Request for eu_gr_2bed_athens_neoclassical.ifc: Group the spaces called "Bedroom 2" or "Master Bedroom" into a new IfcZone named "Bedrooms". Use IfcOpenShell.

First a look at what the model holds.

```python
import ifcopenshell

model = ifcopenshell.open("eu_gr_2bed_athens_neoclassical.ifc")
print(model.schema)
seen = {}
for space in model.by_type("IfcSpace"):
    seen[space.LongName] = seen.get(space.LongName, 0) + 1
for name, count in sorted(seen.items(), key=str):
    print(count, "x", name)
print("zones:", [z.Name for z in model.by_type("IfcZone")][:20])
```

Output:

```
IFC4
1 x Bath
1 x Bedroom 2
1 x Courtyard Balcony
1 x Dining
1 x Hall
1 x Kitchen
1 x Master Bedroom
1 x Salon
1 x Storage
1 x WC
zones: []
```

```python
import ifcopenshell
import ifcopenshell.api.group
import ifcopenshell.api.root

model = ifcopenshell.open("eu_gr_2bed_athens_neoclassical.ifc")

names = {"Bedroom 2", "Master Bedroom"}
spaces = [s for s in model.by_type("IfcSpace") if s.LongName in names]

zone = ifcopenshell.api.root.create_entity(model, ifc_class="IfcZone", name="Bedrooms")
ifcopenshell.api.group.assign_group(model, products=spaces, group=zone)
print(len(spaces), "spaces in", zone.Name)

model.write("eu_gr_2bed_athens_neoclassical_rev.ifc")
```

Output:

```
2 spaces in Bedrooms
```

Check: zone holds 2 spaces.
